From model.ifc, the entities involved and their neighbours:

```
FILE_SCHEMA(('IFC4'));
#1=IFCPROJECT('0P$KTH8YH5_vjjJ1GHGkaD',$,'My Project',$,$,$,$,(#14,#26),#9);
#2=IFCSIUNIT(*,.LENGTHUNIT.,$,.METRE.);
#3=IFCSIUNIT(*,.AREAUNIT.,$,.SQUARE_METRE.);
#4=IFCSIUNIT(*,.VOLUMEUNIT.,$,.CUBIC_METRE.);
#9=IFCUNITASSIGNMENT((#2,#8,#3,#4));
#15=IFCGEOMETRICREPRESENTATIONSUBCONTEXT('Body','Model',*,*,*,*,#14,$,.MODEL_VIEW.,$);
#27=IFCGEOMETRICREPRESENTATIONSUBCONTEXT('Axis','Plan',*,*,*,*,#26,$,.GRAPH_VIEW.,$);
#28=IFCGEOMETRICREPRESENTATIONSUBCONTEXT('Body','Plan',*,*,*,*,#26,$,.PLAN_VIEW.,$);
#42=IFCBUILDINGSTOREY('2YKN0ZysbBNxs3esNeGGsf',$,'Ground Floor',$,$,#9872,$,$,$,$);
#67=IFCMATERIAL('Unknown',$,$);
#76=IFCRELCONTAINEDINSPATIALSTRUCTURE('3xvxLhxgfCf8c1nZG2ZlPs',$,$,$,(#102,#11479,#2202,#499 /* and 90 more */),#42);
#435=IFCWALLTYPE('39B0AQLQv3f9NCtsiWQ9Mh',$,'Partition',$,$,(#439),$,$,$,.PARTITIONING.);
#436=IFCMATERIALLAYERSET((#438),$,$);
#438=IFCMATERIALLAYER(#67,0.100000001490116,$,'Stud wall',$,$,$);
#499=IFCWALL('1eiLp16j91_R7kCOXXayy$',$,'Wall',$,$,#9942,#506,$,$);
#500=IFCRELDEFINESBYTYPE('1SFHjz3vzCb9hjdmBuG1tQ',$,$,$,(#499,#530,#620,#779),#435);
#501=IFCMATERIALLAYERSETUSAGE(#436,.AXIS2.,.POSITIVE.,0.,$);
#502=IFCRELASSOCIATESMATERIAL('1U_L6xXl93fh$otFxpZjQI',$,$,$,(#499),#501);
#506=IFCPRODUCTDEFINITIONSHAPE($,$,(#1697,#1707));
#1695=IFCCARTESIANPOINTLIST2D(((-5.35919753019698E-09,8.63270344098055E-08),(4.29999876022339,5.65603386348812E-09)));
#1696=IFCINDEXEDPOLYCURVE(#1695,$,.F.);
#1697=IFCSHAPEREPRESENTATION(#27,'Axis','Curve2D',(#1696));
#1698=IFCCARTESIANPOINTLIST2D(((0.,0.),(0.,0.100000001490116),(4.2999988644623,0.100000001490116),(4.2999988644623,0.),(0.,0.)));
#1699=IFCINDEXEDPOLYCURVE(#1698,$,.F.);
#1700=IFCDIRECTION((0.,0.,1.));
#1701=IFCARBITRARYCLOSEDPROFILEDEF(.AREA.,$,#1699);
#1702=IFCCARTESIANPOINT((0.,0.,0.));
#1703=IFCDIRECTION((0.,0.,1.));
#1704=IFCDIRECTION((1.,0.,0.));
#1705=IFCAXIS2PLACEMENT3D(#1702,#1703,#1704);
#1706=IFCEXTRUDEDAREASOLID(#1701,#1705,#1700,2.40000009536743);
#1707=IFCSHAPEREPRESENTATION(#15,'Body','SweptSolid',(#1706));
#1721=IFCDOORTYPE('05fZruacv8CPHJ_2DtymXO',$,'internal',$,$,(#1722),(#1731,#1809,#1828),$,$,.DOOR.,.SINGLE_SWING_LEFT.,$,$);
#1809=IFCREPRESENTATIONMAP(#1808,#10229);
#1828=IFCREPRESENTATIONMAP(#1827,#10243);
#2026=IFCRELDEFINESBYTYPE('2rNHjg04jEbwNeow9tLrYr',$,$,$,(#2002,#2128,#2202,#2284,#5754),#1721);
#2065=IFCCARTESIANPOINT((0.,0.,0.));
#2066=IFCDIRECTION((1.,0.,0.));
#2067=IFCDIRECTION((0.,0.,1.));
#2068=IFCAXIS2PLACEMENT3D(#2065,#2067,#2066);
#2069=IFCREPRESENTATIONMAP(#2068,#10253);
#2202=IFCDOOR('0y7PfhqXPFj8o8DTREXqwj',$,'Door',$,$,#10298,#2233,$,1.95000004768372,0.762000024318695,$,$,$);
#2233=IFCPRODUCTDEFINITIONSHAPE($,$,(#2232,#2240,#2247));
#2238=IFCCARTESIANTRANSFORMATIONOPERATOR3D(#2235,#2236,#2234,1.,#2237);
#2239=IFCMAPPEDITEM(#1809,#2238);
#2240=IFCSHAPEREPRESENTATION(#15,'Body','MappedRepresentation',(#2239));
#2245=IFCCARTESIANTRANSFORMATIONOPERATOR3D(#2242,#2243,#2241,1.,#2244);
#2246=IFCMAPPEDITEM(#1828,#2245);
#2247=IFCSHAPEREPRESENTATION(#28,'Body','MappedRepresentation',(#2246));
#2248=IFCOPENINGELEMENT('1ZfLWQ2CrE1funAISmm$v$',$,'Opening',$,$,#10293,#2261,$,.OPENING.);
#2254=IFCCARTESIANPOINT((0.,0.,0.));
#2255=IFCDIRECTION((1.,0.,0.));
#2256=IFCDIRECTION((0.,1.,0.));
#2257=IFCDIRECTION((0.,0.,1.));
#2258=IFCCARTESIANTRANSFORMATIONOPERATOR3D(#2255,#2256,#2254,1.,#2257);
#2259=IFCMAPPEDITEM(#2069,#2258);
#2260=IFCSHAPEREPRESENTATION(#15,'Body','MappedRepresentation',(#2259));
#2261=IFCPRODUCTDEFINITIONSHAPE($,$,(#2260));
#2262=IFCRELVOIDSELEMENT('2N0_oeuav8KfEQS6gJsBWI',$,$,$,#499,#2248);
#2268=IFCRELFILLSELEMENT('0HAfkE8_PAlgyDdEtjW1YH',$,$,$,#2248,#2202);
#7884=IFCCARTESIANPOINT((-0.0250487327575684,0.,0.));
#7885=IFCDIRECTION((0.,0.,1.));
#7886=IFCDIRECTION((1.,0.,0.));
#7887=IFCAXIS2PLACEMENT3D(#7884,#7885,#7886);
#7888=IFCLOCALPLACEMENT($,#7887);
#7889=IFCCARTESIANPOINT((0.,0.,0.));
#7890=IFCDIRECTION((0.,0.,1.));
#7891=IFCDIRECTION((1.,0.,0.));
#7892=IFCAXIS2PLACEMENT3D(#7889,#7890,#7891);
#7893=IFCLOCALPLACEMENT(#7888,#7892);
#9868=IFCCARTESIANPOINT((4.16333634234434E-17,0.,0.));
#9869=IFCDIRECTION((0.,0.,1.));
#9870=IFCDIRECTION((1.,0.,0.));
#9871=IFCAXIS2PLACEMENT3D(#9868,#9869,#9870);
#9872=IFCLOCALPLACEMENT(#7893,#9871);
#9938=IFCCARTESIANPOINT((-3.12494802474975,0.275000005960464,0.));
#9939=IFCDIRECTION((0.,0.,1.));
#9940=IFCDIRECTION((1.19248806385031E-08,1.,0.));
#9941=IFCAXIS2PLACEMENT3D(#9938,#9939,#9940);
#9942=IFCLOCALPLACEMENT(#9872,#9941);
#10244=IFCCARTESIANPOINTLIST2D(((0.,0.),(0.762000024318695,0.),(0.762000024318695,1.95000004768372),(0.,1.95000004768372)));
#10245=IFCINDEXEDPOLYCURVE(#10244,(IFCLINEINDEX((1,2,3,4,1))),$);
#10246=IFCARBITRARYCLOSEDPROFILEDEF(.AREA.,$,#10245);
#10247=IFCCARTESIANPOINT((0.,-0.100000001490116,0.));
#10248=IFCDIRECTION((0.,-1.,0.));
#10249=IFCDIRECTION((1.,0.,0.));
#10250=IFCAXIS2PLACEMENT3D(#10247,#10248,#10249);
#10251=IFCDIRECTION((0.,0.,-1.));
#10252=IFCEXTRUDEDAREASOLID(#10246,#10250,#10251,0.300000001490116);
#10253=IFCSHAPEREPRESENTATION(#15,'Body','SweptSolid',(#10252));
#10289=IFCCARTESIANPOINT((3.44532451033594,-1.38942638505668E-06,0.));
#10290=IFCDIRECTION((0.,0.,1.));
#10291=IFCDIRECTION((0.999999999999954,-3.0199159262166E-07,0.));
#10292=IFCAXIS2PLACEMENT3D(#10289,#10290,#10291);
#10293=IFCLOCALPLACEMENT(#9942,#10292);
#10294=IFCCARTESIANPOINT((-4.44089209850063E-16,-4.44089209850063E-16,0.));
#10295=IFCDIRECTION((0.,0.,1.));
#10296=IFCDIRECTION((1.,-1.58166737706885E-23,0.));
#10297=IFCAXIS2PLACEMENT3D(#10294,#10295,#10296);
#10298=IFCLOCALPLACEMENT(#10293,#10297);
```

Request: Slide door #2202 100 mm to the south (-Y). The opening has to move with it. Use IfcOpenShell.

```python
import ifcopenshell
import ifcopenshell.api.geometry
import ifcopenshell.util.placement
import ifcopenshell.util.unit

model = ifcopenshell.open("model.ifc")
unit_scale = ifcopenshell.util.unit.calculate_unit_scale(model)

door = model.by_id(2202)
opening = door.FillsVoids[0].RelatingOpeningElement
wall = opening.VoidsElements[0].RelatingBuildingElement

wall_matrix = ifcopenshell.util.placement.get_local_placement(wall.ObjectPlacement)
shift = wall_matrix[:3, 0] * -0.1 / unit_scale
before = ifcopenshell.util.placement.get_local_placement(door.ObjectPlacement)[:3, 3].copy()

# The door is placed relative to its opening, so it follows when the opening moves.
matrix = ifcopenshell.util.placement.get_local_placement(opening.ObjectPlacement)
matrix[:3, 3] += shift
ifcopenshell.api.geometry.edit_object_placement(
    model, product=opening, matrix=matrix, is_si=False, should_transform_children=True
)

after = ifcopenshell.util.placement.get_local_placement(door.ObjectPlacement)[:3, 3]
print("door moved by", (after - before).round(3) + 0.0)

model.write("model_rev.ifc")
```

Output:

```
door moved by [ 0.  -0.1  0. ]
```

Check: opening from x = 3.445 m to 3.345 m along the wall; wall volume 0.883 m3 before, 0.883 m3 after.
